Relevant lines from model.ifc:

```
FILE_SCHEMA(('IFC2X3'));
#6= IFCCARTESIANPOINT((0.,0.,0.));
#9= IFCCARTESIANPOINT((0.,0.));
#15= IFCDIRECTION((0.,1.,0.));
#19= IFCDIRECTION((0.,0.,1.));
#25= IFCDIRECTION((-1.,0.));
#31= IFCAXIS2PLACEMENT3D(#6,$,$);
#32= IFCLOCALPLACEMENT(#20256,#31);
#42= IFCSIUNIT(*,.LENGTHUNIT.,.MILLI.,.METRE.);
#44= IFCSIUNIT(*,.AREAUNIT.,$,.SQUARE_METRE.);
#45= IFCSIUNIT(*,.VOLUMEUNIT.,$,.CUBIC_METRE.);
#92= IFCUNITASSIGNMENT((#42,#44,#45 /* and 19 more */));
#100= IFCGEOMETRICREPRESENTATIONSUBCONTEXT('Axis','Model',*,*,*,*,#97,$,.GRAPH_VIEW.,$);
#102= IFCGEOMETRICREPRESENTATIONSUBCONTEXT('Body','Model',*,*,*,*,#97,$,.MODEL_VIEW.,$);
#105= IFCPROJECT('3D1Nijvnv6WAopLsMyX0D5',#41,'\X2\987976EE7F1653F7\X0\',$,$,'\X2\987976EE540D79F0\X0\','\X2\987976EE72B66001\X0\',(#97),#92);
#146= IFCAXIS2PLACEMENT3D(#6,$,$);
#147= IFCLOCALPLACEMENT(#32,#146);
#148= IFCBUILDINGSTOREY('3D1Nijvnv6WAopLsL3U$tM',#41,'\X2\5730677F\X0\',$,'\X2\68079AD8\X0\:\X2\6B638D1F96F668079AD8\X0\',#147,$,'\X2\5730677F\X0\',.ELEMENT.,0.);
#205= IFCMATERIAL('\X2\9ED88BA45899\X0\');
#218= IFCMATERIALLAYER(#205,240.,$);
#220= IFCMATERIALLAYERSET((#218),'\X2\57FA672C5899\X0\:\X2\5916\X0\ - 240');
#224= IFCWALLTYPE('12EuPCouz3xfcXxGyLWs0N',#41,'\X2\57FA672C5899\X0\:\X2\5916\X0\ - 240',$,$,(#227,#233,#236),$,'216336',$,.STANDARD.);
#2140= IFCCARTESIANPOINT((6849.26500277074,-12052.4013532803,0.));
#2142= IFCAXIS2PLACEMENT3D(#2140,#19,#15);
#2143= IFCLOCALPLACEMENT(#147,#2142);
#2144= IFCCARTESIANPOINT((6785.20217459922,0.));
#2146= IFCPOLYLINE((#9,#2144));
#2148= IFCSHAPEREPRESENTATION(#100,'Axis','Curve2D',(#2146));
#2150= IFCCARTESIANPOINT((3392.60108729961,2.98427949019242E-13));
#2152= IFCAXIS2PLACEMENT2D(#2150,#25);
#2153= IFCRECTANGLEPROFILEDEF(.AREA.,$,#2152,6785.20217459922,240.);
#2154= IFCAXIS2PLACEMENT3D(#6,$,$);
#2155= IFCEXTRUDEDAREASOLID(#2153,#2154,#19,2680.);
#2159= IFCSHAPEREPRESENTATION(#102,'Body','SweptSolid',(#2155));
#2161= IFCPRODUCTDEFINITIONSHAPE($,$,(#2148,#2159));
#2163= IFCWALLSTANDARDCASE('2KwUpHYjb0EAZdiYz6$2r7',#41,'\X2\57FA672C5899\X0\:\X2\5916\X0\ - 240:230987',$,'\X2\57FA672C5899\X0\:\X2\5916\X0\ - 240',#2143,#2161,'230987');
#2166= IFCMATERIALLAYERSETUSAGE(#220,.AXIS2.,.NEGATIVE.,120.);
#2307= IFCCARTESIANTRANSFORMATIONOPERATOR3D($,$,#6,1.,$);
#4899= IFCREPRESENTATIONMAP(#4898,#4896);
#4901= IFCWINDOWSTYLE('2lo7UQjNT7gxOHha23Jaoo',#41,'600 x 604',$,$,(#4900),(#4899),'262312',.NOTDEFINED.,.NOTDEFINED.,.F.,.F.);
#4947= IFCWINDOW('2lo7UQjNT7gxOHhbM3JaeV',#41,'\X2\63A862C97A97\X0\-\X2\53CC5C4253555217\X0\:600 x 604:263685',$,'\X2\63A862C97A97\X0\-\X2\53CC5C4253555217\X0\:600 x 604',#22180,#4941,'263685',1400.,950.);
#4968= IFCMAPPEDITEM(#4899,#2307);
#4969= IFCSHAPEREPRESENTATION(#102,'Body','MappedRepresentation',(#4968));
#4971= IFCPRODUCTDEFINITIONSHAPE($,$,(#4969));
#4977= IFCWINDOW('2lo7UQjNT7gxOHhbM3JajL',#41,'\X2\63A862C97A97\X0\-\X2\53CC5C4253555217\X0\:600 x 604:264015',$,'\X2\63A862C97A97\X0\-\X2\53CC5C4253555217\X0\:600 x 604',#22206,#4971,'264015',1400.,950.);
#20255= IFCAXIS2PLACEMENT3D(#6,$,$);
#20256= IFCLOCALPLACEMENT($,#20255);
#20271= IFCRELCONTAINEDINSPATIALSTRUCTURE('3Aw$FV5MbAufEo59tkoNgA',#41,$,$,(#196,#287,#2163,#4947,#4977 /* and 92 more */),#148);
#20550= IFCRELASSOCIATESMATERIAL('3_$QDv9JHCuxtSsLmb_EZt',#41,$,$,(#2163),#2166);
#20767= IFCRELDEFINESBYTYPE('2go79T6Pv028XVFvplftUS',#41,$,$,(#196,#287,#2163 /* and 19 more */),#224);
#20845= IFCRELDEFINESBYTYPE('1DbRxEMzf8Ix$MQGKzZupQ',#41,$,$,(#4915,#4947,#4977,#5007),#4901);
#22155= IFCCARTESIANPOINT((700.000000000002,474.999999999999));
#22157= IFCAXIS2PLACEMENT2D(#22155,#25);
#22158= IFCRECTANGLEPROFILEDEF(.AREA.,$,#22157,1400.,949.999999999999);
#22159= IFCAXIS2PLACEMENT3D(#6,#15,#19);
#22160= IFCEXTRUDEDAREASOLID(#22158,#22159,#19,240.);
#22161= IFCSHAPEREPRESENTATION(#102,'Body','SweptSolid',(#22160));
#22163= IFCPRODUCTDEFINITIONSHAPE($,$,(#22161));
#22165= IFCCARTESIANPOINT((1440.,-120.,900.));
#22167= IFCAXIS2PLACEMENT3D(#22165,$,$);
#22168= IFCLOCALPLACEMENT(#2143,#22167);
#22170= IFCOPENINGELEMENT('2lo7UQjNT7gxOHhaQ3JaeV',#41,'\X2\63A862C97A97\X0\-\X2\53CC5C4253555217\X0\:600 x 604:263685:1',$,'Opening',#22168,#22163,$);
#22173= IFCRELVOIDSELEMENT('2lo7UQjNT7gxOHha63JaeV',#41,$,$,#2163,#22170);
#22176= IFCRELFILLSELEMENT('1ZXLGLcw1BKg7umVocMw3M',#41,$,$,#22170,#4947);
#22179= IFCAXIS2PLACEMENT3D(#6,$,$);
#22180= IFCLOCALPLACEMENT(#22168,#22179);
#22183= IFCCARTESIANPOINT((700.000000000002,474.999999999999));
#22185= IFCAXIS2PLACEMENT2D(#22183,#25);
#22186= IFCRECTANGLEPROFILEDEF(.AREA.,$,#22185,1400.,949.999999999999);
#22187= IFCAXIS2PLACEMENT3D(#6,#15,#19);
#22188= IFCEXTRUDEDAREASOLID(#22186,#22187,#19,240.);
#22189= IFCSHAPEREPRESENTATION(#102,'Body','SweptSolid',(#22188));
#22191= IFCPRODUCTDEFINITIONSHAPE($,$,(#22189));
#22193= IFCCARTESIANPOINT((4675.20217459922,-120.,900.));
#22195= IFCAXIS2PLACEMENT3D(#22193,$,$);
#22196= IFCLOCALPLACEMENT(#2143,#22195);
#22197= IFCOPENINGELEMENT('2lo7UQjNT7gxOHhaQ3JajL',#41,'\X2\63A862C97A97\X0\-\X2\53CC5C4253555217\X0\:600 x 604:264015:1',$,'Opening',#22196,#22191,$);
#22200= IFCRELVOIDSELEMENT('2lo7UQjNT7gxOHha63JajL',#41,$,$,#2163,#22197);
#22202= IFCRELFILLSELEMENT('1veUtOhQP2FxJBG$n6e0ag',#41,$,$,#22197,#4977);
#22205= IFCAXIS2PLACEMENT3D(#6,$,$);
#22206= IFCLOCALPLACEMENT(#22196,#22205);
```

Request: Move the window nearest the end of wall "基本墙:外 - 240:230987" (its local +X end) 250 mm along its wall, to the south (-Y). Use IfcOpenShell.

```python
import ifcopenshell
import ifcopenshell.api.geometry
import ifcopenshell.util.placement

model = ifcopenshell.open("model.ifc")

window = model.by_guid("2lo7UQjNT7gxOHhbM3JajL")
opening = window.FillsVoids[0].RelatingOpeningElement
wall = opening.VoidsElements[0].RelatingBuildingElement

wall_matrix = ifcopenshell.util.placement.get_local_placement(wall.ObjectPlacement)
shift = wall_matrix[:3, 0] * -250.0
before = ifcopenshell.util.placement.get_local_placement(window.ObjectPlacement)[:3, 3].copy()

# The window is placed relative to its opening, so it follows when the opening moves.
matrix = ifcopenshell.util.placement.get_local_placement(opening.ObjectPlacement)
matrix[:3, 3] += shift
ifcopenshell.api.geometry.edit_object_placement(
    model, product=opening, matrix=matrix, is_si=False, should_transform_children=True
)

after = ifcopenshell.util.placement.get_local_placement(window.ObjectPlacement)[:3, 3]
print("window moved by", (after - before).round(3) + 0.0)

model.write("model_rev.ifc")
```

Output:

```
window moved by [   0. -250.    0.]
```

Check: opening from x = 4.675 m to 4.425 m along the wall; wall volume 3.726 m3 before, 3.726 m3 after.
